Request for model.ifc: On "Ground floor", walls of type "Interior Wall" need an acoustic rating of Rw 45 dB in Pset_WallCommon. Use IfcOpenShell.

First a look at what the model holds.

```python
import ifcopenshell
import ifcopenshell.util.element

model = ifcopenshell.open("model.ifc")
print(model.schema)
storey = next(s for s in model.by_type("IfcBuildingStorey") if s.Name == "Ground floor")
walls = [e for e in ifcopenshell.util.element.get_decomposition(storey) if e.is_a("IfcWall")]
seen = {}
for e in walls:
    element_type = ifcopenshell.util.element.get_type(e)
    key = (element_type.Name if element_type != e and element_type else None, ifcopenshell.util.element.get_pset(e, "Pset_WallCommon", "AcousticRating"))
    seen[key] = seen.get(key, 0) + 1
for (name, value), count in sorted(seen.items(), key=str):
    print(count, "x", name, "|", value)
```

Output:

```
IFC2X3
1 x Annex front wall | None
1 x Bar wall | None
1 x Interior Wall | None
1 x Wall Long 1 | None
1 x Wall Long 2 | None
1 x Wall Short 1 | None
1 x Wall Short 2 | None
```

```python
import ifcopenshell
import ifcopenshell.api.pset
import ifcopenshell.util.element

model = ifcopenshell.open("model.ifc")

storey = next(s for s in model.by_type("IfcBuildingStorey") if s.Name == "Ground floor")
walls = [e for e in ifcopenshell.util.element.get_decomposition(storey) if e.is_a("IfcWall")]

count = 0
for e in walls:
    element_type = ifcopenshell.util.element.get_type(e)
    if element_type in (None, e) or element_type.Name != "Interior Wall":
        continue
    # add_pset returns the element's existing set when there is one.
    pset = ifcopenshell.api.pset.add_pset(model, product=e, name="Pset_WallCommon")
    ifcopenshell.api.pset.edit_pset(model, pset=pset, properties={"AcousticRating": "Rw 45 dB"})
    count += 1

print(count, "walls updated")

model.write("model_edited.ifc")
```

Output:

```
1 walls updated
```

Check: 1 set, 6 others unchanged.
